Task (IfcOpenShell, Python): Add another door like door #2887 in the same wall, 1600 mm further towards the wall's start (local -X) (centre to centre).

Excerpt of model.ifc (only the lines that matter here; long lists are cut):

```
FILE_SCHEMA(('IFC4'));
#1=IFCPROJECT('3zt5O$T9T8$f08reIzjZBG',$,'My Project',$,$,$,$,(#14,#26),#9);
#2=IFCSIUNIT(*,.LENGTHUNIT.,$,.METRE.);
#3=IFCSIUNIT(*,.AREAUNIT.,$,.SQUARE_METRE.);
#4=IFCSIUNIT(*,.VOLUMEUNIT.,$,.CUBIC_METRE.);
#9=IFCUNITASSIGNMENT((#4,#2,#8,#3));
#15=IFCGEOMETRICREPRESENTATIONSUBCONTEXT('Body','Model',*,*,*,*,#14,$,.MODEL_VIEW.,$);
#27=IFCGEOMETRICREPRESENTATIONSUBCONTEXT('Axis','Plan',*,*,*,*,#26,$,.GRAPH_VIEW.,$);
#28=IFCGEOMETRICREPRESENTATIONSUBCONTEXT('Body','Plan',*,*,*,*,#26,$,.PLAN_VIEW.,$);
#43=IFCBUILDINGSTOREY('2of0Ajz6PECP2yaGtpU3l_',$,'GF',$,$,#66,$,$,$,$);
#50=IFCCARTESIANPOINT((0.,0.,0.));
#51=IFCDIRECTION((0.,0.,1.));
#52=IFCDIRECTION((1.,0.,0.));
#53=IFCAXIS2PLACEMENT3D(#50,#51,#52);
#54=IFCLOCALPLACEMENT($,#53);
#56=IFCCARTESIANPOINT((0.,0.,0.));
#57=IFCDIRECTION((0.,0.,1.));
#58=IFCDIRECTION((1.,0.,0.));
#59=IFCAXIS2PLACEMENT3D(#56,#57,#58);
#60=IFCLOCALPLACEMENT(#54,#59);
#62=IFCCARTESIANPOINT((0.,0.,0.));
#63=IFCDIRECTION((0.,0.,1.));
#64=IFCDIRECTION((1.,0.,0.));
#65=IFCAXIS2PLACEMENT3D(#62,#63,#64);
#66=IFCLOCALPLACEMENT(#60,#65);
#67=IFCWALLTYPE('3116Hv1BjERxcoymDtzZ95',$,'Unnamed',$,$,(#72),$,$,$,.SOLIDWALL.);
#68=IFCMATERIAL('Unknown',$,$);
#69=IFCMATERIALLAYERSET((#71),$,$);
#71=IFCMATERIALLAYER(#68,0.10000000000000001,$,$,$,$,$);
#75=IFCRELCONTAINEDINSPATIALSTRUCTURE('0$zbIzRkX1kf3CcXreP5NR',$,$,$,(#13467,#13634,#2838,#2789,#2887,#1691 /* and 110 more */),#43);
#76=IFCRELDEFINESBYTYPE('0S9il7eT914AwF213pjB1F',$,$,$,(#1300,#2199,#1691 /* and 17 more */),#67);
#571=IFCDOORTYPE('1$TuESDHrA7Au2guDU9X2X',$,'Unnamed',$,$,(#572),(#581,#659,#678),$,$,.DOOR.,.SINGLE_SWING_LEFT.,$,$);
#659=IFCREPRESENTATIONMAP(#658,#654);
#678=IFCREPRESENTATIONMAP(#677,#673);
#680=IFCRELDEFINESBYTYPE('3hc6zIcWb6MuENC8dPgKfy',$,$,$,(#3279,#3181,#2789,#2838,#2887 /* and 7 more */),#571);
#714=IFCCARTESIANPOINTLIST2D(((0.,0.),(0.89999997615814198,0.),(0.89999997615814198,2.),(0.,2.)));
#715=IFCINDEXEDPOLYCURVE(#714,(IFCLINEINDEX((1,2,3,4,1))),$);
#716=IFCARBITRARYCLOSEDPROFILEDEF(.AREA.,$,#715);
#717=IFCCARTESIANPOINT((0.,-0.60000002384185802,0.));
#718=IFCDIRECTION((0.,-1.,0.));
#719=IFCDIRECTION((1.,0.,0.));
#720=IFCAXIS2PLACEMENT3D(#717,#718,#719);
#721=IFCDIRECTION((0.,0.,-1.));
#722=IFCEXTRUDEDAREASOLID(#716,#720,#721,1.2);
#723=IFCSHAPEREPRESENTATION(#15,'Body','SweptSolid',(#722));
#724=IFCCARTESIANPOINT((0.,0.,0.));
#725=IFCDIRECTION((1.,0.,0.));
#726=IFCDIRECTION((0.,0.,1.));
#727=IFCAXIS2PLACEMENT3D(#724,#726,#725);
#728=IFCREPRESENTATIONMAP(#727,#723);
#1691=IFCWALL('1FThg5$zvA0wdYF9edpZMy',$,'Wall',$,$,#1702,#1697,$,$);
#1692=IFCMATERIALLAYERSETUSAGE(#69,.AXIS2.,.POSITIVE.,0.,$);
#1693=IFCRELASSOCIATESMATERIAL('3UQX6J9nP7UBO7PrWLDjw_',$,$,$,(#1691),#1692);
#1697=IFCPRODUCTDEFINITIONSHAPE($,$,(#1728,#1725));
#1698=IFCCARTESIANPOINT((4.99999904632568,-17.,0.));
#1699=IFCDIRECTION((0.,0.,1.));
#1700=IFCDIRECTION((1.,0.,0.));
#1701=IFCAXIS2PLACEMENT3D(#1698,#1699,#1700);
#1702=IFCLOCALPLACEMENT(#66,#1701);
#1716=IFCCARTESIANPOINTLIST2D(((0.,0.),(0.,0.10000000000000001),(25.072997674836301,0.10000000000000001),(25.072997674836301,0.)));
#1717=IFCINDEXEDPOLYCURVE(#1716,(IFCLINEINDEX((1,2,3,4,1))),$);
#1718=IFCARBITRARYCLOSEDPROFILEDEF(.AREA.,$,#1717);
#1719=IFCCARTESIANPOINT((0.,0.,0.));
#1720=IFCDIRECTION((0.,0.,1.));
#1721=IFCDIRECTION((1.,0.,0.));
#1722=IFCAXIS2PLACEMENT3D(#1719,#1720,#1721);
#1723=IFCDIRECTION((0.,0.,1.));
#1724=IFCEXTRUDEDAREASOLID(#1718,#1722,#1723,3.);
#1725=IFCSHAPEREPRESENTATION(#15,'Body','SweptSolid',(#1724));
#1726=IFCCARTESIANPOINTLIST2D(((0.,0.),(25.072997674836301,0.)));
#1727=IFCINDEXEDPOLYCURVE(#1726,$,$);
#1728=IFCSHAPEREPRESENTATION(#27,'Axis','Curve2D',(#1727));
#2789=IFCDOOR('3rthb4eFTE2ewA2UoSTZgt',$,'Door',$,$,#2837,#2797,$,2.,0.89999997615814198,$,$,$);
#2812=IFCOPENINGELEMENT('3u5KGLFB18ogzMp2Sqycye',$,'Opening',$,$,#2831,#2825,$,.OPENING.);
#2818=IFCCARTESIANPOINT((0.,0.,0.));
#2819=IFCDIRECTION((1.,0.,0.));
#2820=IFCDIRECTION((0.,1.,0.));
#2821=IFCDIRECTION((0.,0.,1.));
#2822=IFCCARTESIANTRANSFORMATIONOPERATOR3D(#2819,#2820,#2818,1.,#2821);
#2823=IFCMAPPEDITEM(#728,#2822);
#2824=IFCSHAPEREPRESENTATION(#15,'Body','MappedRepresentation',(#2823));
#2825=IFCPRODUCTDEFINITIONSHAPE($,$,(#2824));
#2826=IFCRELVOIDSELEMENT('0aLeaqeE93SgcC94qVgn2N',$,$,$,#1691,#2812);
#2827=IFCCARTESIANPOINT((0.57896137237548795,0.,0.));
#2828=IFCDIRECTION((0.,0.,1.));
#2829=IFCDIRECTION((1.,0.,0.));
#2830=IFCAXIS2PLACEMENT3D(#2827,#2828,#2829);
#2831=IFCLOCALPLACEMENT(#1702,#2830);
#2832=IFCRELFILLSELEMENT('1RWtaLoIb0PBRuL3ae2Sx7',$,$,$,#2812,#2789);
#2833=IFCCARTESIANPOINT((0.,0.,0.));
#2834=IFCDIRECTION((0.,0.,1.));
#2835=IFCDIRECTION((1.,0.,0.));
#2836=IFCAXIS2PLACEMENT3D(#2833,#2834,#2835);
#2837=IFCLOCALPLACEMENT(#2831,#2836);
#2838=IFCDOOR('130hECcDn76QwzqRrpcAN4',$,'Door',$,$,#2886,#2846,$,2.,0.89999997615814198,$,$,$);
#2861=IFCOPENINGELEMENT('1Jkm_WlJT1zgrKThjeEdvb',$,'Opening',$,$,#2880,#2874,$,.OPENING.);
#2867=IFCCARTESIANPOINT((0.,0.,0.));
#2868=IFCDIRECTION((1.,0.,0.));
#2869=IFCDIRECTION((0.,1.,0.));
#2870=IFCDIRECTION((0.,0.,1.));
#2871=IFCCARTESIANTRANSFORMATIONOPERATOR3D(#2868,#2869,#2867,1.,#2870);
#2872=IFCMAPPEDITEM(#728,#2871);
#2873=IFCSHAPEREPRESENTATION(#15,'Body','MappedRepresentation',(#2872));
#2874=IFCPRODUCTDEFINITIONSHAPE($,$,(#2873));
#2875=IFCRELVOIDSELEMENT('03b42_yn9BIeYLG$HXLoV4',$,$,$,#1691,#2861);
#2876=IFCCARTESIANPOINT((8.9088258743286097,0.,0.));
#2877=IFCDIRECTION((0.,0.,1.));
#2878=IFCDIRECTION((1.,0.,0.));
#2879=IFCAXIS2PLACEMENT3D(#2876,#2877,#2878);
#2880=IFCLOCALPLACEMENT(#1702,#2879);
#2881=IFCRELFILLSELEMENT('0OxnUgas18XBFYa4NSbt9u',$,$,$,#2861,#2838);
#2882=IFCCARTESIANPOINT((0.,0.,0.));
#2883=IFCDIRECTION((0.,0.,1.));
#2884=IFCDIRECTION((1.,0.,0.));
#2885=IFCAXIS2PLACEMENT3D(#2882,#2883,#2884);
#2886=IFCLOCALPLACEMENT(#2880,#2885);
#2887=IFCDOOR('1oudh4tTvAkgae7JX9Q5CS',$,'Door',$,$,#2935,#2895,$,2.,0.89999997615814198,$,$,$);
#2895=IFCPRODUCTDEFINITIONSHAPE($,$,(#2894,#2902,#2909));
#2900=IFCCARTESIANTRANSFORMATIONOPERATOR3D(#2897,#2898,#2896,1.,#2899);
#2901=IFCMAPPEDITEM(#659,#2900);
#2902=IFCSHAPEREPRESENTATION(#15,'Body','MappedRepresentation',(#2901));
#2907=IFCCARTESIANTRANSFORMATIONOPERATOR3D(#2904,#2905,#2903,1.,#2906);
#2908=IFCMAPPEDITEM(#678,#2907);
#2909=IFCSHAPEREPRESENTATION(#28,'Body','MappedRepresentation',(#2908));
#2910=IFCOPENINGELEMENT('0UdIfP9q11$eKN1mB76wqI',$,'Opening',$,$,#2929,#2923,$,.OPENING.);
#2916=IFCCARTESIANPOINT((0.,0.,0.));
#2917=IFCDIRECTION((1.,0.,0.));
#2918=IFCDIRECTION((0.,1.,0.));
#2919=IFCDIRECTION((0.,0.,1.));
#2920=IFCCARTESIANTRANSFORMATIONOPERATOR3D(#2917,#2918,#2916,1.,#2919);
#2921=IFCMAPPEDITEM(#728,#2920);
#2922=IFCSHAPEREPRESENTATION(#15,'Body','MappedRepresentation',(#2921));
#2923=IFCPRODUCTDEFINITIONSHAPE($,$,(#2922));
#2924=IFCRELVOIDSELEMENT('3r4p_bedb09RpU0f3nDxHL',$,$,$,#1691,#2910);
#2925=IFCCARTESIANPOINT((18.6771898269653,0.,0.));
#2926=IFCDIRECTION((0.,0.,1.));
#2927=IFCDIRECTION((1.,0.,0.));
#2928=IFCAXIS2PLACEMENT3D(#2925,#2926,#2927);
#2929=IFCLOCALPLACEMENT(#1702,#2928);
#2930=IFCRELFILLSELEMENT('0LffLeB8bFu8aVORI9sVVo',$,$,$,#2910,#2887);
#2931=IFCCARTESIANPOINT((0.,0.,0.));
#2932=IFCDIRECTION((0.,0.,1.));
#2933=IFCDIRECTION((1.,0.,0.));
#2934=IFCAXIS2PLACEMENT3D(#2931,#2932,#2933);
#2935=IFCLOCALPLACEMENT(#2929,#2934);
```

```python
import ifcopenshell
import ifcopenshell.api.feature
import ifcopenshell.api.geometry
import ifcopenshell.api.root
import ifcopenshell.geom
import ifcopenshell.util.element
import ifcopenshell.util.placement
import ifcopenshell.util.shape

model = ifcopenshell.open("model.ifc")
settings = ifcopenshell.geom.settings()


def volume(element):
    """Net volume in cubic metres, openings subtracted."""
    shape = ifcopenshell.geom.create_shape(settings, element)
    return ifcopenshell.util.shape.get_volume(shape.geometry)


door = model.by_guid("1oudh4tTvAkgae7JX9Q5CS")
opening = door.FillsVoids[0].RelatingOpeningElement
wall = opening.VoidsElements[0].RelatingBuildingElement
before = volume(wall)
shift = ifcopenshell.util.placement.get_local_placement(wall.ObjectPlacement)[:3, 0] * -1.6

# copy_class copies the void relationship, type, container and properties, but no geometry.
new_opening = ifcopenshell.api.root.copy_class(model, product=opening)
new_opening.Representation = ifcopenshell.util.element.copy_deep(
    model, opening.Representation, exclude=["IfcGeometricRepresentationContext", "IfcRepresentationMap"]
)
new_door = ifcopenshell.api.root.copy_class(model, product=door)
new_door.Representation = ifcopenshell.util.element.copy_deep(
    model, door.Representation, exclude=["IfcGeometricRepresentationContext", "IfcRepresentationMap"]
)
ifcopenshell.api.feature.add_filling(model, opening=new_opening, element=new_door)

for old, new in ((opening, new_opening), (door, new_door)):
    matrix = ifcopenshell.util.placement.get_local_placement(old.ObjectPlacement)
    matrix[:3, 3] += shift
    ifcopenshell.api.geometry.edit_object_placement(model, product=new, matrix=matrix, is_si=False)

after = volume(wall)

print(f"wall volume {before:.3f} -> {after:.3f} m3")

model.write("model_rev.ifc")
```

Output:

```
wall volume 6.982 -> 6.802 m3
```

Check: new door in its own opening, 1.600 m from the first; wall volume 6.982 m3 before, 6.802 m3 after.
